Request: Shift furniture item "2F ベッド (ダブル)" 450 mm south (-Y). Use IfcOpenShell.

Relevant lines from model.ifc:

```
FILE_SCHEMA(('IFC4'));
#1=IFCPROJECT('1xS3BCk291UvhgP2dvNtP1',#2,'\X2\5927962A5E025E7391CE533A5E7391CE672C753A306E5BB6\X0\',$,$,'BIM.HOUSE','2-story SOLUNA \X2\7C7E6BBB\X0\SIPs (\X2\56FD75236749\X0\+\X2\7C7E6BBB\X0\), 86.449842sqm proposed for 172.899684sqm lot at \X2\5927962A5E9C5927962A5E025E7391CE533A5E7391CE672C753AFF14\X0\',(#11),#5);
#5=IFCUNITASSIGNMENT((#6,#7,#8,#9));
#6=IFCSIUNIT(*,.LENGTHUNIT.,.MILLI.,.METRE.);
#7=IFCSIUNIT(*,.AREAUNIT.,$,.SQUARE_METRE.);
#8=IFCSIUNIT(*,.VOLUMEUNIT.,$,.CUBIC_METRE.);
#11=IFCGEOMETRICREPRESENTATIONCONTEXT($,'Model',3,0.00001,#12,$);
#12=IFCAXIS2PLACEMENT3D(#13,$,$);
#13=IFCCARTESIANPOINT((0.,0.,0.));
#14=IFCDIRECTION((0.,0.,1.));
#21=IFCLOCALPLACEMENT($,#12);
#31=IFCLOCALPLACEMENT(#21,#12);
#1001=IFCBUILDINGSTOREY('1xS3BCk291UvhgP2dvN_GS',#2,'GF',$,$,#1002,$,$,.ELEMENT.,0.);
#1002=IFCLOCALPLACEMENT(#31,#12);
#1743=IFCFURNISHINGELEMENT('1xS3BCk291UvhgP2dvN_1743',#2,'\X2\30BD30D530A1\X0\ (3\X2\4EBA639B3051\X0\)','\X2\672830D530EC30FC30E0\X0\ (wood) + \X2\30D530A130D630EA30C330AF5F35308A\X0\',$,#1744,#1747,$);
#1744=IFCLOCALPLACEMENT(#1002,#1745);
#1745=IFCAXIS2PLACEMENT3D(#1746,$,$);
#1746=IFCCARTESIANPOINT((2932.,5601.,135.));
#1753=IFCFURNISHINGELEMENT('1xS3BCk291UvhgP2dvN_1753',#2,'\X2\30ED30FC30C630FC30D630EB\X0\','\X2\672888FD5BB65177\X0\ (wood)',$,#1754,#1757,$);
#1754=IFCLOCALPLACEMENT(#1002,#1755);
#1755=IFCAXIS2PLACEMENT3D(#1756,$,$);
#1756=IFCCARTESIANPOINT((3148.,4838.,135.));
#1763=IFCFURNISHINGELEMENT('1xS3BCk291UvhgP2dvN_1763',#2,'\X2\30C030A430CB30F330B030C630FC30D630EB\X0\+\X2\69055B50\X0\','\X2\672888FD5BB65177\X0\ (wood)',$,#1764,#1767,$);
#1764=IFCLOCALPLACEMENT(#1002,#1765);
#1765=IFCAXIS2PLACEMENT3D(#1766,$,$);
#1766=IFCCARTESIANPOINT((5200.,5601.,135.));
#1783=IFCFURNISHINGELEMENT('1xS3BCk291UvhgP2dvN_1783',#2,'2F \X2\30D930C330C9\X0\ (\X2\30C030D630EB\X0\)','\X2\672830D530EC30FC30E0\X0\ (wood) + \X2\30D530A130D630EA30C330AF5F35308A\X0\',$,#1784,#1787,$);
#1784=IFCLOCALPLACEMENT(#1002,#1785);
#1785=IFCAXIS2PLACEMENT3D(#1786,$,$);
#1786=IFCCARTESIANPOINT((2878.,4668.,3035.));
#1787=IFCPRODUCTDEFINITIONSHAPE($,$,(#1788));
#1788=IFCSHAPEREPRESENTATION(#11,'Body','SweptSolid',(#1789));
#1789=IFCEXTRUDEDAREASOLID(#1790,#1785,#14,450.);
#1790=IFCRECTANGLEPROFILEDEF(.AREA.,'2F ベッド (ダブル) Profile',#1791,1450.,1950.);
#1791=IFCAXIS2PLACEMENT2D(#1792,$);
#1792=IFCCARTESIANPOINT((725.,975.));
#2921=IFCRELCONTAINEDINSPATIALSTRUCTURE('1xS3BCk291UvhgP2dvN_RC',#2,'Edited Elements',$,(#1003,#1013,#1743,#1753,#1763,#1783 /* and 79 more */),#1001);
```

```python
import ifcopenshell
import ifcopenshell.api.geometry
import ifcopenshell.util.placement
import ifcopenshell.util.unit

model = ifcopenshell.open("model.ifc")
unit_scale = ifcopenshell.util.unit.calculate_unit_scale(model)

item = model.by_id(1783)
matrix = ifcopenshell.util.placement.get_local_placement(item.ObjectPlacement)
matrix[1, 3] -= 0.45 / unit_scale
ifcopenshell.api.geometry.edit_object_placement(model, product=item, matrix=matrix, is_si=False)

print(ifcopenshell.util.placement.get_local_placement(item.ObjectPlacement).round(3) + 0.0)

model.write("model_edited.ifc")
```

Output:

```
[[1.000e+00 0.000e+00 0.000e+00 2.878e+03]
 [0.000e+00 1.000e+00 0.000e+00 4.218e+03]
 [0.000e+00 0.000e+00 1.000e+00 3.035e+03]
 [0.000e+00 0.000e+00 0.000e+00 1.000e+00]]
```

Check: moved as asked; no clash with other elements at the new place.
